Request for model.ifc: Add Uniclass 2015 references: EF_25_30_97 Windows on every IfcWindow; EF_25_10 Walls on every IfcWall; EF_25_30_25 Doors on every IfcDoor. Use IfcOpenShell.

First a look at what the model holds.

```python
import ifcopenshell

model = ifcopenshell.open("model.ifc")
print(model.schema)
print("classifications:", [c.Name for c in model.by_type("IfcClassification")])
for ifc_class in ("IfcDoor", "IfcRoof", "IfcStair", "IfcWall", "IfcWindow"):
    print(ifc_class, len(model.by_type(ifc_class)))
```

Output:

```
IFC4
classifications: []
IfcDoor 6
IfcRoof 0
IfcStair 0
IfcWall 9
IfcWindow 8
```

```python
import ifcopenshell
import ifcopenshell.api.classification

model = ifcopenshell.open("model.ifc")

system = ifcopenshell.api.classification.add_classification(model, classification="Uniclass 2015")

codes = {
    "IfcWindow": ("EF_25_30_97", "Windows"),
    "IfcWall": ("EF_25_10", "Walls"),
    "IfcDoor": ("EF_25_30_25", "Doors"),
}
for ifc_class, (code, name) in codes.items():
    products = model.by_type(ifc_class)
    ifcopenshell.api.classification.add_reference(
        model, products=products, classification=system, identification=code, name=name
    )
    print(code, len(products))

model.write("model_updated.ifc")
```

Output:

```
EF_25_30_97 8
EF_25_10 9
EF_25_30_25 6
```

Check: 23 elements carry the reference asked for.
